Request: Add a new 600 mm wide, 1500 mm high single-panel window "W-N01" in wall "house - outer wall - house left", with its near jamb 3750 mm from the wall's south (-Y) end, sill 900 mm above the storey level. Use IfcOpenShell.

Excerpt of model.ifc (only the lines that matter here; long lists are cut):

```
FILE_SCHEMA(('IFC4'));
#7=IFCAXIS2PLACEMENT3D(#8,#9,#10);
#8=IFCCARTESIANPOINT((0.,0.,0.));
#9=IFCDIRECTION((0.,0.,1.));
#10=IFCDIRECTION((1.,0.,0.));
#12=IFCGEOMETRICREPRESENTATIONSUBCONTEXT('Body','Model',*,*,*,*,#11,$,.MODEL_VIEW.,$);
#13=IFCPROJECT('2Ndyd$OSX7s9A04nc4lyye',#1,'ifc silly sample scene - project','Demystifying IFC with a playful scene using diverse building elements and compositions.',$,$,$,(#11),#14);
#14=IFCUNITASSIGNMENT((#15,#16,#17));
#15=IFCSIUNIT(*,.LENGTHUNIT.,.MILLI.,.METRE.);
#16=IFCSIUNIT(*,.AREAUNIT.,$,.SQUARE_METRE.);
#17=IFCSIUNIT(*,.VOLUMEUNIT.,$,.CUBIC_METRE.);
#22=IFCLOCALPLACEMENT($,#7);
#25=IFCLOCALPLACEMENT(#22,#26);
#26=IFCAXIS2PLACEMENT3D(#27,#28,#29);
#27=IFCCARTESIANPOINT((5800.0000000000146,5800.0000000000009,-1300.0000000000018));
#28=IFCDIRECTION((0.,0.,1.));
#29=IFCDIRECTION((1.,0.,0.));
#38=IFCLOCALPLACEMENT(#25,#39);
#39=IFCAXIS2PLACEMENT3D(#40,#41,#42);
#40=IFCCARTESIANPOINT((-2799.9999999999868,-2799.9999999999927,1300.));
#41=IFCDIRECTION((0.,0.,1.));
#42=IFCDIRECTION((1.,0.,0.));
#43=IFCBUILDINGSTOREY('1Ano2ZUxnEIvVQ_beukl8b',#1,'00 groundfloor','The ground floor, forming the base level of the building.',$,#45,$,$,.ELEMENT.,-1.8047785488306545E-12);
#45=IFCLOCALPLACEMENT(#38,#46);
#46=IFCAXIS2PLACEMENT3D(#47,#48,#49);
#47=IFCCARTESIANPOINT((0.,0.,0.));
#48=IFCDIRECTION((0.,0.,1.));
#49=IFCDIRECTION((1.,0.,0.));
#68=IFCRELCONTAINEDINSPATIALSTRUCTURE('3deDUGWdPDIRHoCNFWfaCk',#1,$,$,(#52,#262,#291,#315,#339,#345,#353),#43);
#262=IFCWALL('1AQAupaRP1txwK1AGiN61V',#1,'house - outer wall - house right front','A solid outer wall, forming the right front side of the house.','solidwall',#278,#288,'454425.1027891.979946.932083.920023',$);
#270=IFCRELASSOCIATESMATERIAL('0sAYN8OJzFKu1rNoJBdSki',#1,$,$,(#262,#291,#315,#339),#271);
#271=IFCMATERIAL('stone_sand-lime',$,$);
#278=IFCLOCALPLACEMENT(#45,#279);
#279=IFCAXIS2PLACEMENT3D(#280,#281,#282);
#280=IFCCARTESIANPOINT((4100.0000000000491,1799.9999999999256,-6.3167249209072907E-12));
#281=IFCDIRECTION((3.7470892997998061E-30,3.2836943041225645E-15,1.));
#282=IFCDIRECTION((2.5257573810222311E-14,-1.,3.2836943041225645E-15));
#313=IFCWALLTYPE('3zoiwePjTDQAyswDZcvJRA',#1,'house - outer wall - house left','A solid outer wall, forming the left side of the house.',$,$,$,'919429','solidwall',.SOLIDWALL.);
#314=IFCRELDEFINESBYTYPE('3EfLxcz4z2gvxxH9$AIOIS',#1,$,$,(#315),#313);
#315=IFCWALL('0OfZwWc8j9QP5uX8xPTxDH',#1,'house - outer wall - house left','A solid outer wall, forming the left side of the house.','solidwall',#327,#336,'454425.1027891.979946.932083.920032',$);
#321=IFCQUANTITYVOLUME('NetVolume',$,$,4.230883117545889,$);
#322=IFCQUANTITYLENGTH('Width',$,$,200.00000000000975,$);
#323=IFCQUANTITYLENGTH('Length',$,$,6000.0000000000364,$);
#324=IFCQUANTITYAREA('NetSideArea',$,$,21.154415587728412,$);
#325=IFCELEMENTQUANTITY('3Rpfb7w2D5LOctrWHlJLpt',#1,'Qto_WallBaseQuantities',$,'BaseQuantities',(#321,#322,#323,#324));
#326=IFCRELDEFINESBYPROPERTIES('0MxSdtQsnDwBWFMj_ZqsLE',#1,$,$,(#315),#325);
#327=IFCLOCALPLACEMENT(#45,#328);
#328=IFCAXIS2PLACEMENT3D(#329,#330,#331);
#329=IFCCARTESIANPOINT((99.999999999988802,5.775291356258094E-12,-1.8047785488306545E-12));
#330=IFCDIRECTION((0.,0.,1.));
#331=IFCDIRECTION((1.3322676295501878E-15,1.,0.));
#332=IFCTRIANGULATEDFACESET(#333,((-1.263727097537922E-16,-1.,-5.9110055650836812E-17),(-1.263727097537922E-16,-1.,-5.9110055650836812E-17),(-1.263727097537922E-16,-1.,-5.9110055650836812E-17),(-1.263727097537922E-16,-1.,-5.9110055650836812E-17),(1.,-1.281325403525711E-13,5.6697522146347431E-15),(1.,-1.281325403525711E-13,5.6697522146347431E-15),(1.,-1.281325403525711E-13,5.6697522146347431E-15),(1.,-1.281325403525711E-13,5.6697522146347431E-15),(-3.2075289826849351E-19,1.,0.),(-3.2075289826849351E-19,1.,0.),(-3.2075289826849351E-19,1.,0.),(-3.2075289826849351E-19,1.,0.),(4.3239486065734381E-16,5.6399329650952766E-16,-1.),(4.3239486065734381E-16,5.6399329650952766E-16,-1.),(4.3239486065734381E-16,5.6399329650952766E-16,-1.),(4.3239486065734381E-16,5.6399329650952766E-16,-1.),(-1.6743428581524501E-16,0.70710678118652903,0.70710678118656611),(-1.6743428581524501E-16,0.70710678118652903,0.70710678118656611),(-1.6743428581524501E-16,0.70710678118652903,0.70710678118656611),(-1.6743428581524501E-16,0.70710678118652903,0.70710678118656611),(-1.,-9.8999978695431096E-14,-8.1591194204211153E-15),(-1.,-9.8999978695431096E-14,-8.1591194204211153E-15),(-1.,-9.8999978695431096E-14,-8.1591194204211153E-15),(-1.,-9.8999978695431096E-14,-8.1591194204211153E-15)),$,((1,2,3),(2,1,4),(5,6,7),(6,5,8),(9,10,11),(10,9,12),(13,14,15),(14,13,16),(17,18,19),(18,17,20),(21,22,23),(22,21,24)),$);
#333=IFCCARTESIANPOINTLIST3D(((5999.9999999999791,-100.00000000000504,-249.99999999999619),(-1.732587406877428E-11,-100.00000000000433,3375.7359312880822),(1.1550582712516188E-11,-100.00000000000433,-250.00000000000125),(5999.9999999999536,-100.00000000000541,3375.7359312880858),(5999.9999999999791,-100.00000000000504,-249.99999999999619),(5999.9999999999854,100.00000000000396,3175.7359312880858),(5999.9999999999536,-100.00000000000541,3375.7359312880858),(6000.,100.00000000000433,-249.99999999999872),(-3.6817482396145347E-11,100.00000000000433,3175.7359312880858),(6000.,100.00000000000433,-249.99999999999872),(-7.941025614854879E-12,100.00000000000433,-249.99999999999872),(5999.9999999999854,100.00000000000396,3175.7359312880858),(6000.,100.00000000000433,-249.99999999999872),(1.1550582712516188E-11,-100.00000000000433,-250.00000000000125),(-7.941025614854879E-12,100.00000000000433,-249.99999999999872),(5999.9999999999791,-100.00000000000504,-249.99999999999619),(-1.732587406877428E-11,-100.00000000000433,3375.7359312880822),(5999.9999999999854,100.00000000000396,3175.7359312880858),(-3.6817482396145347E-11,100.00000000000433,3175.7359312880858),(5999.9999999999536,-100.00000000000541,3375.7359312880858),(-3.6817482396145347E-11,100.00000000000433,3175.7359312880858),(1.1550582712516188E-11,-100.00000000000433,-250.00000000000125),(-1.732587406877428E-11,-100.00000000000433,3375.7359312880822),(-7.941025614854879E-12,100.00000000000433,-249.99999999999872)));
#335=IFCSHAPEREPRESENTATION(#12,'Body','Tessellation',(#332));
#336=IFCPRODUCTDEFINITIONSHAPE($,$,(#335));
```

```python
import numpy as np
import ifcopenshell
import ifcopenshell.api.feature
import ifcopenshell.api.geometry
import ifcopenshell.api.pset
import ifcopenshell.api.root
import ifcopenshell.api.spatial
import ifcopenshell.geom
import ifcopenshell.util.element
import ifcopenshell.util.placement
import ifcopenshell.util.representation
import ifcopenshell.util.shape
import ifcopenshell.util.unit

model = ifcopenshell.open("model.ifc")
unit_scale = ifcopenshell.util.unit.calculate_unit_scale(model)
area_scale = ifcopenshell.util.unit.calculate_unit_scale(model, "AREAUNIT")
volume_scale = ifcopenshell.util.unit.calculate_unit_scale(model, "VOLUMEUNIT")
settings = ifcopenshell.geom.settings()


def volume(element):
    """Net volume in cubic metres, openings subtracted."""
    shape = ifcopenshell.geom.create_shape(settings, element)
    return ifcopenshell.util.shape.get_volume(shape.geometry)


wall = model.by_guid("0OfZwWc8j9QP5uX8xPTxDH")
storey = ifcopenshell.util.element.get_container(wall, ifc_class="IfcBuildingStorey")
context = ifcopenshell.util.representation.get_context(model, "Model", "Body", "MODEL_VIEW")
before = volume(wall)

width, height, from_end, sill = 0.6, 1.5, 3.75, 0.9  # metres

# The wall runs along its own X axis, and the end named is its -X end.
wall_shape = ifcopenshell.geom.create_shape(settings, wall)
x, y, z = ifcopenshell.util.shape.get_vertices(wall_shape.geometry).T
start = x.min() + from_end
face, thickness = float(y.min()), float(y.max() - y.min())
wall_matrix = ifcopenshell.util.placement.get_local_placement(wall.ObjectPlacement)
level = ifcopenshell.util.placement.get_local_placement(storey.ObjectPlacement)[2, 3]


def in_wall(x, y):
    """Placement at x, y metres in the wall's axes, at sill height."""
    matrix = wall_matrix.copy()
    matrix[:, 3] = wall_matrix @ np.array([x / unit_scale, y / unit_scale, 0.0, 1.0])
    matrix[2, 3] = level + sill / unit_scale
    return matrix


# Opening: a box that overshoots both wall faces by 50 mm.
opening = ifcopenshell.api.root.create_entity(model, ifc_class="IfcOpeningElement", predefined_type="OPENING")
box = ifcopenshell.api.geometry.add_wall_representation(
    model, context=context, length=width, height=height, thickness=thickness + 0.1
)
ifcopenshell.api.geometry.assign_representation(model, product=opening, representation=box)
ifcopenshell.api.geometry.edit_object_placement(model, product=opening, matrix=in_wall(start, face - 0.05), is_si=False)
ifcopenshell.api.feature.add_feature(model, feature=opening, element=wall)

window = ifcopenshell.api.root.create_entity(model, ifc_class="IfcWindow", name="W-N01", predefined_type="WINDOW")
window.OverallWidth, window.OverallHeight = width / unit_scale, height / unit_scale
window.PartitioningType = "SINGLE_PANEL"
body = ifcopenshell.api.geometry.add_window_representation(
    model,
    context=context,
    overall_width=window.OverallWidth,
    overall_height=window.OverallHeight,
    partition_type="SINGLE_PANEL",
)
ifcopenshell.api.geometry.assign_representation(model, product=window, representation=body)
ifcopenshell.api.spatial.assign_container(model, products=[window], relating_structure=storey)
ifcopenshell.api.feature.add_filling(model, opening=opening, element=window)

# Centre the window in the wall's thickness.
ifcopenshell.api.geometry.edit_object_placement(model, product=window, matrix=in_wall(start, face), is_si=False)
window_shape = ifcopenshell.geom.create_shape(settings, window)
depth = ifcopenshell.util.shape.get_vertices(window_shape.geometry)[:, 1]
offset = face + thickness / 2 - (depth.min() + depth.max()) / 2
ifcopenshell.api.geometry.edit_object_placement(model, product=window, matrix=in_wall(start, offset), is_si=False)

after = volume(wall)

# Update the wall's stored quantities.
qto = model.by_id(ifcopenshell.util.element.get_pset(wall, "Qto_WallBaseQuantities", should_inherit=False)["id"])
ifcopenshell.api.pset.edit_qto(model, qto=qto, properties={
    "NetVolume": after / volume_scale,
    "NetSideArea": after / thickness / area_scale,
})

print(f"wall volume {before:.3f} -> {after:.3f} m3")

model.write("model_rev.ifc")
```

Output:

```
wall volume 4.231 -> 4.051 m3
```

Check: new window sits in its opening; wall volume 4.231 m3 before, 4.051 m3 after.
